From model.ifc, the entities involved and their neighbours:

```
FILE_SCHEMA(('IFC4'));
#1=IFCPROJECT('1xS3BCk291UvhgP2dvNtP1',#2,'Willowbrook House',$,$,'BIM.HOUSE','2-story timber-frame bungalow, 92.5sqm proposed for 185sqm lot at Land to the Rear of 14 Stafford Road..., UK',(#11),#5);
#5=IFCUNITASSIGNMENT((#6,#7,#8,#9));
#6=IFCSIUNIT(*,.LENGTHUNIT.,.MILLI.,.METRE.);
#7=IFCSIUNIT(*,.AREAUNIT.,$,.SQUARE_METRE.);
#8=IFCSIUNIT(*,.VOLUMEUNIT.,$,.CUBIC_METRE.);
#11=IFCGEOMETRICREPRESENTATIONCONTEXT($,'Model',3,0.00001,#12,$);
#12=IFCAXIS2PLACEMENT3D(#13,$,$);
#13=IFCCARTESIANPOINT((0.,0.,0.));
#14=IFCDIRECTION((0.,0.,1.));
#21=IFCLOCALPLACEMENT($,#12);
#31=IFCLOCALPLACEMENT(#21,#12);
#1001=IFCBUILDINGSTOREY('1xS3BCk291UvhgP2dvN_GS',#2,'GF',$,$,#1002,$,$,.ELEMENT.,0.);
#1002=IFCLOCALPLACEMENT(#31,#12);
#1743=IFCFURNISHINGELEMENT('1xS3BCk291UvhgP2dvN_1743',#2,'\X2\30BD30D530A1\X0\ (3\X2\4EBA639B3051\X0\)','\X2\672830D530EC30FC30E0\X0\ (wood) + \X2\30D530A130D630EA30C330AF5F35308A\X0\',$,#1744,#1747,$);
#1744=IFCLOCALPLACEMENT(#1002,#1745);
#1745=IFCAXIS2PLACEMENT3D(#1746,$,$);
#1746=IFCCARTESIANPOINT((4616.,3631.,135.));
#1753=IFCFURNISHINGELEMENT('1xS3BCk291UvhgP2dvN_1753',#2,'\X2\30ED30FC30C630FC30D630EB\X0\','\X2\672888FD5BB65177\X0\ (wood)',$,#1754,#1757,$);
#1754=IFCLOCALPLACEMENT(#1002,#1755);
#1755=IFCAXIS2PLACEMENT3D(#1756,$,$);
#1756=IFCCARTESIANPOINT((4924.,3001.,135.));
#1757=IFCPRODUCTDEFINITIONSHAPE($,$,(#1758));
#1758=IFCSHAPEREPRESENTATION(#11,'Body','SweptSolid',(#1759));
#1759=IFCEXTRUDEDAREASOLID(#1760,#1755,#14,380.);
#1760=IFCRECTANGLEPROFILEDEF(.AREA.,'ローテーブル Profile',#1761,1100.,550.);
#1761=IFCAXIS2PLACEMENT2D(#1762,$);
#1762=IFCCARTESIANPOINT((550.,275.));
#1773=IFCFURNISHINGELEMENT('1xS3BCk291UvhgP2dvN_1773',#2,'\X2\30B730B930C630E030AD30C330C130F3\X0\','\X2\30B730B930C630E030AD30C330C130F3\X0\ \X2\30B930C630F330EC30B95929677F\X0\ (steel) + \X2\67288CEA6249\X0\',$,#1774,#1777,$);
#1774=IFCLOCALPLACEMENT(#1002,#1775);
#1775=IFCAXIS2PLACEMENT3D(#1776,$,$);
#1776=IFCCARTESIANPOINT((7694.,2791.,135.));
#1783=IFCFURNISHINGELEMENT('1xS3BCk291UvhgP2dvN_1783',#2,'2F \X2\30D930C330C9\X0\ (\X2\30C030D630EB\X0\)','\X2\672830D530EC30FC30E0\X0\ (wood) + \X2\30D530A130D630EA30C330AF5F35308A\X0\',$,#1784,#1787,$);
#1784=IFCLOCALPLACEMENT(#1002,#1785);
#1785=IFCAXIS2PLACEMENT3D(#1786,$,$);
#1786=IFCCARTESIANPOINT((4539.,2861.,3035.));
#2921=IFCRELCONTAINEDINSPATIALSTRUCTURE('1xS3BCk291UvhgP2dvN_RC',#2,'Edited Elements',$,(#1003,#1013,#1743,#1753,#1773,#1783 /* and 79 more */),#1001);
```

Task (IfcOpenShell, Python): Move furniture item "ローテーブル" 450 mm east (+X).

```python
import ifcopenshell
import ifcopenshell.api.geometry
import ifcopenshell.util.placement
import ifcopenshell.util.unit

model = ifcopenshell.open("model.ifc")
unit_scale = ifcopenshell.util.unit.calculate_unit_scale(model)

item = model.by_guid("1xS3BCk291UvhgP2dvN_1753")
matrix = ifcopenshell.util.placement.get_local_placement(item.ObjectPlacement)
matrix[0, 3] += 0.45 / unit_scale
ifcopenshell.api.geometry.edit_object_placement(model, product=item, matrix=matrix, is_si=False)

print(ifcopenshell.util.placement.get_local_placement(item.ObjectPlacement).round(3) + 0.0)

model.write("model_rev.ifc")
```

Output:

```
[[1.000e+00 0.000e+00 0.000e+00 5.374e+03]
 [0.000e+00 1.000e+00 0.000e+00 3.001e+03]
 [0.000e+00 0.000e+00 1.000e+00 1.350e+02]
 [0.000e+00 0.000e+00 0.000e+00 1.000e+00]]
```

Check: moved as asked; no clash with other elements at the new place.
